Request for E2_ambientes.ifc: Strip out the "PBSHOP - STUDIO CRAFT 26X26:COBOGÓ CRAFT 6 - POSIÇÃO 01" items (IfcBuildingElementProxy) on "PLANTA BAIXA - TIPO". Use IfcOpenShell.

First a look at what the model holds.

```python
import ifcopenshell
import ifcopenshell.util.element

model = ifcopenshell.open("E2_ambientes.ifc")
print(model.schema)
storey = next(s for s in model.by_type("IfcBuildingStorey") if s.Name == "PLANTA BAIXA - TIPO")
proxies = [e for e in ifcopenshell.util.element.get_decomposition(storey) if e.is_a("IfcBuildingElementProxy")]
seen = {}
for e in proxies:
    element_type = ifcopenshell.util.element.get_type(e)
    name = element_type.Name if element_type not in (None, e) else None
    seen[name] = seen.get(name, 0) + 1
for name, count in sorted(seen.items(), key=str):
    print(count, "x", name)
```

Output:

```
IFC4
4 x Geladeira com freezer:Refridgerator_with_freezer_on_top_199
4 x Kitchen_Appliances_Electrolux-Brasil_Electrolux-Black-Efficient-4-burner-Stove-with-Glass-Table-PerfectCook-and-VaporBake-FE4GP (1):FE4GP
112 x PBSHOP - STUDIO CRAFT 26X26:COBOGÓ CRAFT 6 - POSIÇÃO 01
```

```python
import ifcopenshell
import ifcopenshell.api.root
import ifcopenshell.util.element

model = ifcopenshell.open("E2_ambientes.ifc")

storey = next(s for s in model.by_type("IfcBuildingStorey") if s.Name == "PLANTA BAIXA - TIPO")
proxies = [e for e in ifcopenshell.util.element.get_decomposition(storey) if e.is_a("IfcBuildingElementProxy")]
targets = [e for e in proxies if (t := ifcopenshell.util.element.get_type(e)) not in (None, e) and t.Name == "PBSHOP - STUDIO CRAFT 26X26:COBOGÓ CRAFT 6 - POSIÇÃO 01"]

for e in targets:
    ifcopenshell.api.root.remove_product(model, product=e)
print(len(targets), "removed")

model.write("E2_ambientes_rev.ifc")
```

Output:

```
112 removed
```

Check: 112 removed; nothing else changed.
